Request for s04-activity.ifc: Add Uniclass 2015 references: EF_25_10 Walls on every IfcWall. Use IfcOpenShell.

First a look at what the model holds.

```python
import ifcopenshell

model = ifcopenshell.open("s04-activity.ifc")
print(model.schema)
print("classifications:", [c.Name for c in model.by_type("IfcClassification")])
for ifc_class in ("IfcDoor", "IfcRoof", "IfcStair", "IfcWall", "IfcWindow"):
    print(ifc_class, len(model.by_type(ifc_class)))
```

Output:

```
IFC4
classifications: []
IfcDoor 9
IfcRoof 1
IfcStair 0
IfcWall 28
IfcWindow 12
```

```python
import ifcopenshell
import ifcopenshell.api.classification

model = ifcopenshell.open("s04-activity.ifc")

system = ifcopenshell.api.classification.add_classification(model, classification="Uniclass 2015")

codes = {
    "IfcWall": ("EF_25_10", "Walls"),
}
for ifc_class, (code, name) in codes.items():
    products = model.by_type(ifc_class)
    ifcopenshell.api.classification.add_reference(
        model, products=products, classification=system, identification=code, name=name
    )
    print(code, len(products))

model.write("s04-activity_edited.ifc")
```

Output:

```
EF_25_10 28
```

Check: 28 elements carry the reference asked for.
